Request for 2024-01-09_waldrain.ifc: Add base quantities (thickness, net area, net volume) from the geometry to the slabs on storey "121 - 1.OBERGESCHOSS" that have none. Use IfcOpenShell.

First a look at what the model holds.

```python
import ifcopenshell
import ifcopenshell.util.element
import ifcopenshell.util.unit

model = ifcopenshell.open("2024-01-09_waldrain.ifc")
print(model.schema)
for unit_type in ("LENGTHUNIT", "AREAUNIT", "VOLUMEUNIT"):
    print(unit_type, ifcopenshell.util.unit.calculate_unit_scale(model, unit_type))
storey = next(s for s in model.by_type("IfcBuildingStorey") if s.Name == "121 - 1.OBERGESCHOSS")
slabs = [e for e in ifcopenshell.util.element.get_decomposition(storey) if e.is_a("IfcSlab")]
for e in sorted(slabs, key=lambda e: e.id()):
    print(e.id(), e.is_a(), e.Name, list(ifcopenshell.util.element.get_psets(e, qtos_only=True)), sep=" | ")
```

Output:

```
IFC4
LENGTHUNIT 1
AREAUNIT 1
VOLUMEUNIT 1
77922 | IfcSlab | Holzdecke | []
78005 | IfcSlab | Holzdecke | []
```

```python
import ifcopenshell
import ifcopenshell.api.pset
import ifcopenshell.geom
import ifcopenshell.util.element
import ifcopenshell.util.shape
import ifcopenshell.util.unit

model = ifcopenshell.open("2024-01-09_waldrain.ifc")
unit_scale = ifcopenshell.util.unit.calculate_unit_scale(model)
area_scale = ifcopenshell.util.unit.calculate_unit_scale(model, "AREAUNIT")
volume_scale = ifcopenshell.util.unit.calculate_unit_scale(model, "VOLUMEUNIT")
settings = ifcopenshell.geom.settings()

storey = next(s for s in model.by_type("IfcBuildingStorey") if s.Name == "121 - 1.OBERGESCHOSS")
slabs = [e for e in ifcopenshell.util.element.get_decomposition(storey) if e.is_a("IfcSlab")]

for e in sorted(slabs, key=lambda e: e.id()):
    if ifcopenshell.util.element.get_psets(e, qtos_only=True, should_inherit=False):
        continue
    # Geometry comes back in metres, in the element's own axes.
    shape = ifcopenshell.geom.create_shape(settings, e)
    values = {
        "Width": ifcopenshell.util.shape.get_z(shape.geometry) / unit_scale,
        "NetArea": ifcopenshell.util.shape.get_footprint_area(shape.geometry) / area_scale,
        "NetVolume": ifcopenshell.util.shape.get_volume(shape.geometry) / volume_scale,
    }
    qto = ifcopenshell.api.pset.add_qto(model, product=e, name="Qto_SlabBaseQuantities")
    ifcopenshell.api.pset.edit_qto(model, qto=qto, properties=values)
    print(e.id(), {k: round(v, 3) for k, v in values.items()})

model.write("2024-01-09_waldrain_rev.ifc")
```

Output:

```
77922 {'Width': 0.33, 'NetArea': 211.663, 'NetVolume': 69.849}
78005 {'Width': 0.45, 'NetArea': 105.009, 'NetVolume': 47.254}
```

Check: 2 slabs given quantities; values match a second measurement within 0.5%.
